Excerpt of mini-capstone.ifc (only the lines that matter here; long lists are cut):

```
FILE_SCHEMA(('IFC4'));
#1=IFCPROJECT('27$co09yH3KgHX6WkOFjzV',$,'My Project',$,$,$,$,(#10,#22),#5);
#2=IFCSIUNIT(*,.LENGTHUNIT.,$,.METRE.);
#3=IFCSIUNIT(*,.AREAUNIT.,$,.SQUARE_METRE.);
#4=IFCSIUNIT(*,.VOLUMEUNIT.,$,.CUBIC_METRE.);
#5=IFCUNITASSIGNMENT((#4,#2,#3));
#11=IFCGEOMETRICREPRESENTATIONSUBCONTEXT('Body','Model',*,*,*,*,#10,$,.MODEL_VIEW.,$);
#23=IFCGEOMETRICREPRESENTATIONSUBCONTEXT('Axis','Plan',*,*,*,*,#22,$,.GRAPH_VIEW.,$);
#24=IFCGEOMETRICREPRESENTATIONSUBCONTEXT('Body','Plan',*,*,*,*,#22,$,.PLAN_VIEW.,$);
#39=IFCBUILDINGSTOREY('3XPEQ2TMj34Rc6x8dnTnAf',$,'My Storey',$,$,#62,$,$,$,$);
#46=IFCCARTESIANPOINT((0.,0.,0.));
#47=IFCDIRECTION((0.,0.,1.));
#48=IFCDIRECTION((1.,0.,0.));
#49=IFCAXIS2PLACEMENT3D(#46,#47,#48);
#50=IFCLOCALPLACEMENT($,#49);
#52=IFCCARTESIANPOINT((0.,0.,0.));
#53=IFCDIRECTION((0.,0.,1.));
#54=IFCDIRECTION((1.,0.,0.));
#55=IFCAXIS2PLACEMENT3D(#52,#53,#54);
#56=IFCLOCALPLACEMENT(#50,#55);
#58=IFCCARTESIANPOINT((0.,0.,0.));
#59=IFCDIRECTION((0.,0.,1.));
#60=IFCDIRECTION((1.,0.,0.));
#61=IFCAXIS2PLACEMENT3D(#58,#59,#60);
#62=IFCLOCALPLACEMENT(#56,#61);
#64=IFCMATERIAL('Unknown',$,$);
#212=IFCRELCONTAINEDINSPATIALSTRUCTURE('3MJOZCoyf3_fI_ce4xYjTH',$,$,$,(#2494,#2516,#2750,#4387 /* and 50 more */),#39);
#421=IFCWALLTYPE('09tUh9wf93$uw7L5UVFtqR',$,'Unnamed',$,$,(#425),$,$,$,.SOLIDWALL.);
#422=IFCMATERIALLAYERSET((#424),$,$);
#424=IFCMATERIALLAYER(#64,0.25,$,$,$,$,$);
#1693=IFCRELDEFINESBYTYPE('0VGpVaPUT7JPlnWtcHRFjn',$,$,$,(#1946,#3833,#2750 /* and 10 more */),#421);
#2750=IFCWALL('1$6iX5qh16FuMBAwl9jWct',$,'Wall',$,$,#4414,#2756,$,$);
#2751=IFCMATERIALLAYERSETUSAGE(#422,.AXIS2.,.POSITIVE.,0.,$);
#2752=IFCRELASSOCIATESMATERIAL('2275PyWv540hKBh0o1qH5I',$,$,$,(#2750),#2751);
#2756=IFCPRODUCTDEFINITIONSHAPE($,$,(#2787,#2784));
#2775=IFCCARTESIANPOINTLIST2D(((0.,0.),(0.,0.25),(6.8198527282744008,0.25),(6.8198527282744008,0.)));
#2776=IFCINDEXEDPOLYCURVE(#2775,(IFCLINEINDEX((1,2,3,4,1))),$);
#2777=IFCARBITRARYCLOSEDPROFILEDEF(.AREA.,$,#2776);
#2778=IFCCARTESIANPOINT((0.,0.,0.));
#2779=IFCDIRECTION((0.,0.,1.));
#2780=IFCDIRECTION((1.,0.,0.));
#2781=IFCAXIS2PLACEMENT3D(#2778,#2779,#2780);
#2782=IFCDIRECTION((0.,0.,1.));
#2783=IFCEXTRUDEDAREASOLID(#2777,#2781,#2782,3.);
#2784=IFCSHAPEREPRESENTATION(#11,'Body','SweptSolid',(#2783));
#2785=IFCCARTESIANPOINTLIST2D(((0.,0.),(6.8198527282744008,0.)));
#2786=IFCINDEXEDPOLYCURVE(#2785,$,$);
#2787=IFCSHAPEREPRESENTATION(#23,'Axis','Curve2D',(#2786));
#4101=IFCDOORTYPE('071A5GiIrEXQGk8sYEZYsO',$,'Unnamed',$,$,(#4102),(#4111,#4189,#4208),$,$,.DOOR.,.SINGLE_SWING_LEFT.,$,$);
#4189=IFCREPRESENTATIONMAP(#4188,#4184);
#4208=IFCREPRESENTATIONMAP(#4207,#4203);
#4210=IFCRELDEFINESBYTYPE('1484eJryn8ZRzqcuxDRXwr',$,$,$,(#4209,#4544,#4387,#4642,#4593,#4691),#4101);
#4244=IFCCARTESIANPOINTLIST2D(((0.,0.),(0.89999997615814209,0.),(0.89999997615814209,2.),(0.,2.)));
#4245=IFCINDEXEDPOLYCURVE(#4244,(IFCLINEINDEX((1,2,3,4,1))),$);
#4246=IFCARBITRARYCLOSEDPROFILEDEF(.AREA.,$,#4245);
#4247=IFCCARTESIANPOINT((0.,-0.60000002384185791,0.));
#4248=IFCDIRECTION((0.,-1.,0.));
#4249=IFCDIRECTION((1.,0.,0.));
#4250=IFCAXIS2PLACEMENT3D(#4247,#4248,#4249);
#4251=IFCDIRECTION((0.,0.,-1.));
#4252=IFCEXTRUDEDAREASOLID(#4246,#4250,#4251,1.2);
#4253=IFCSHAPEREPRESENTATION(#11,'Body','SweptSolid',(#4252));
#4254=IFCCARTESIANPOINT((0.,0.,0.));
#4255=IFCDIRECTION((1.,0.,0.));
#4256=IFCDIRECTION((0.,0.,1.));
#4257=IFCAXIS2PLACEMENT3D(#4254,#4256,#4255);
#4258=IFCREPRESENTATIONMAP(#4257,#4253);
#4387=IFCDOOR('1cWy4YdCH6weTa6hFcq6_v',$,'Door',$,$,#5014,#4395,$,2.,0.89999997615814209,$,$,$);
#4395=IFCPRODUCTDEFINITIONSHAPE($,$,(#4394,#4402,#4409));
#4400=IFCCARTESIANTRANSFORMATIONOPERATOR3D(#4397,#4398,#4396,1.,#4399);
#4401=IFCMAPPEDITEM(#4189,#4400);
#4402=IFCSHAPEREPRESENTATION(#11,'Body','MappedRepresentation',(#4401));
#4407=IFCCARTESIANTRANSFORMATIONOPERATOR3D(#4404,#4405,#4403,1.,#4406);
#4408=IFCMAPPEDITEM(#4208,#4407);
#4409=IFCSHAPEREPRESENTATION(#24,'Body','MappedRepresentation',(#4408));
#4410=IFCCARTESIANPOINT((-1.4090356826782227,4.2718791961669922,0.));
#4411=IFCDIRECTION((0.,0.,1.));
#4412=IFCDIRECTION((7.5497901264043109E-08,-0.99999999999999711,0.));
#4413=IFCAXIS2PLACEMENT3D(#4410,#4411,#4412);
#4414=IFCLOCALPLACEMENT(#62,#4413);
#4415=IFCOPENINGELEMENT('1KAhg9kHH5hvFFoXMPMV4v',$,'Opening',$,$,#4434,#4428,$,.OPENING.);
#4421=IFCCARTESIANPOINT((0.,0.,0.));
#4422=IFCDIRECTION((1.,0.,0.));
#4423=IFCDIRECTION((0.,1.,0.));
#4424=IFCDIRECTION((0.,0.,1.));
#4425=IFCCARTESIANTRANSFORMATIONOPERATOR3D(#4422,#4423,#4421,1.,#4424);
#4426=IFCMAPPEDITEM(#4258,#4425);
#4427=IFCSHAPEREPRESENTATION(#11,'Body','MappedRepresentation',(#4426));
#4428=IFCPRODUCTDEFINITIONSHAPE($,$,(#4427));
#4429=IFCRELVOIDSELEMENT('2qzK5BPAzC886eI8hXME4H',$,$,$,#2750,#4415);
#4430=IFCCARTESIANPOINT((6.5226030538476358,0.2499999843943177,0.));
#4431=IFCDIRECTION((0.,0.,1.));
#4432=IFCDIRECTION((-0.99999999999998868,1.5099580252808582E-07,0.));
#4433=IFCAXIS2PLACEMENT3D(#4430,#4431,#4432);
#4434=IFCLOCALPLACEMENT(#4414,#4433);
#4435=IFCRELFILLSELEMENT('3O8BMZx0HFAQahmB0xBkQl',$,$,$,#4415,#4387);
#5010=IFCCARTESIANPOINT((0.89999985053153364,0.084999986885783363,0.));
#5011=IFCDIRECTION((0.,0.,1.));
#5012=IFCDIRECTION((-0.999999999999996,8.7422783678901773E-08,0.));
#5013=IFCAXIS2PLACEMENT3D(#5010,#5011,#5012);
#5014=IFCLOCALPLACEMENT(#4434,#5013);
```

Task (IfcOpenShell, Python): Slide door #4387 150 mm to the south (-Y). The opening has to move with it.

```python
import ifcopenshell
import ifcopenshell.api.geometry
import ifcopenshell.util.placement

model = ifcopenshell.open("mini-capstone.ifc")

door = model.by_guid("1cWy4YdCH6weTa6hFcq6_v")
opening = door.FillsVoids[0].RelatingOpeningElement
wall = opening.VoidsElements[0].RelatingBuildingElement

wall_matrix = ifcopenshell.util.placement.get_local_placement(wall.ObjectPlacement)
shift = wall_matrix[:3, 0] * 0.15
before = ifcopenshell.util.placement.get_local_placement(door.ObjectPlacement)[:3, 3].copy()

# The door is placed relative to its opening, so it follows when the opening moves.
matrix = ifcopenshell.util.placement.get_local_placement(opening.ObjectPlacement)
matrix[:3, 3] += shift
ifcopenshell.api.geometry.edit_object_placement(
    model, product=opening, matrix=matrix, is_si=False, should_transform_children=True
)

after = ifcopenshell.util.placement.get_local_placement(door.ObjectPlacement)[:3, 3]
print("door moved by", (after - before).round(3) + 0.0)

model.write("mini-capstone_edited.ifc")
```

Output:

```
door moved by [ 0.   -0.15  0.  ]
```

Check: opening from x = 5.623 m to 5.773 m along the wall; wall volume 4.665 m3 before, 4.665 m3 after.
